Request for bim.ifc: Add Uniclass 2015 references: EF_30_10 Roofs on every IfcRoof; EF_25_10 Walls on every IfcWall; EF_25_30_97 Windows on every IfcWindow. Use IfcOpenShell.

First a look at what the model holds.

```python
import ifcopenshell

model = ifcopenshell.open("bim.ifc")
print(model.schema)
print("classifications:", [c.Name for c in model.by_type("IfcClassification")])
for ifc_class in ("IfcDoor", "IfcRoof", "IfcStair", "IfcWall", "IfcWindow"):
    print(ifc_class, len(model.by_type(ifc_class)))
```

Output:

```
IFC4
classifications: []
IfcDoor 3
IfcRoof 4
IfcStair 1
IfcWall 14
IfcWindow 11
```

```python
import ifcopenshell
import ifcopenshell.api.classification

model = ifcopenshell.open("bim.ifc")

system = ifcopenshell.api.classification.add_classification(model, classification="Uniclass 2015")

codes = {
    "IfcRoof": ("EF_30_10", "Roofs"),
    "IfcWall": ("EF_25_10", "Walls"),
    "IfcWindow": ("EF_25_30_97", "Windows"),
}
for ifc_class, (code, name) in codes.items():
    products = model.by_type(ifc_class)
    ifcopenshell.api.classification.add_reference(
        model, products=products, classification=system, identification=code, name=name
    )
    print(code, len(products))

model.write("bim-out.ifc")
```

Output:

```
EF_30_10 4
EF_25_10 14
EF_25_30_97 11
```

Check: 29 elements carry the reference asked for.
